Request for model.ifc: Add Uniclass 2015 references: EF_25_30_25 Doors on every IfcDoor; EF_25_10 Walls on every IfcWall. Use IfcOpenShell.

First a look at what the model holds.

```python
import ifcopenshell

model = ifcopenshell.open("model.ifc")
print(model.schema)
print("classifications:", [c.Name for c in model.by_type("IfcClassification")])
for ifc_class in ("IfcDoor", "IfcRoof", "IfcStair", "IfcWall", "IfcWindow"):
    print(ifc_class, len(model.by_type(ifc_class)))
```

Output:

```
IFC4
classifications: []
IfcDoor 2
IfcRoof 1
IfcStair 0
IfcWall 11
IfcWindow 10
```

```python
import ifcopenshell
import ifcopenshell.api.classification

model = ifcopenshell.open("model.ifc")

system = ifcopenshell.api.classification.add_classification(model, classification="Uniclass 2015")

codes = {
    "IfcDoor": ("EF_25_30_25", "Doors"),
    "IfcWall": ("EF_25_10", "Walls"),
}
for ifc_class, (code, name) in codes.items():
    products = model.by_type(ifc_class)
    ifcopenshell.api.classification.add_reference(
        model, products=products, classification=system, identification=code, name=name
    )
    print(code, len(products))

model.write("model-out.ifc")
```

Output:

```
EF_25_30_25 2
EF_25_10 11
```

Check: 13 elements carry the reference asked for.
